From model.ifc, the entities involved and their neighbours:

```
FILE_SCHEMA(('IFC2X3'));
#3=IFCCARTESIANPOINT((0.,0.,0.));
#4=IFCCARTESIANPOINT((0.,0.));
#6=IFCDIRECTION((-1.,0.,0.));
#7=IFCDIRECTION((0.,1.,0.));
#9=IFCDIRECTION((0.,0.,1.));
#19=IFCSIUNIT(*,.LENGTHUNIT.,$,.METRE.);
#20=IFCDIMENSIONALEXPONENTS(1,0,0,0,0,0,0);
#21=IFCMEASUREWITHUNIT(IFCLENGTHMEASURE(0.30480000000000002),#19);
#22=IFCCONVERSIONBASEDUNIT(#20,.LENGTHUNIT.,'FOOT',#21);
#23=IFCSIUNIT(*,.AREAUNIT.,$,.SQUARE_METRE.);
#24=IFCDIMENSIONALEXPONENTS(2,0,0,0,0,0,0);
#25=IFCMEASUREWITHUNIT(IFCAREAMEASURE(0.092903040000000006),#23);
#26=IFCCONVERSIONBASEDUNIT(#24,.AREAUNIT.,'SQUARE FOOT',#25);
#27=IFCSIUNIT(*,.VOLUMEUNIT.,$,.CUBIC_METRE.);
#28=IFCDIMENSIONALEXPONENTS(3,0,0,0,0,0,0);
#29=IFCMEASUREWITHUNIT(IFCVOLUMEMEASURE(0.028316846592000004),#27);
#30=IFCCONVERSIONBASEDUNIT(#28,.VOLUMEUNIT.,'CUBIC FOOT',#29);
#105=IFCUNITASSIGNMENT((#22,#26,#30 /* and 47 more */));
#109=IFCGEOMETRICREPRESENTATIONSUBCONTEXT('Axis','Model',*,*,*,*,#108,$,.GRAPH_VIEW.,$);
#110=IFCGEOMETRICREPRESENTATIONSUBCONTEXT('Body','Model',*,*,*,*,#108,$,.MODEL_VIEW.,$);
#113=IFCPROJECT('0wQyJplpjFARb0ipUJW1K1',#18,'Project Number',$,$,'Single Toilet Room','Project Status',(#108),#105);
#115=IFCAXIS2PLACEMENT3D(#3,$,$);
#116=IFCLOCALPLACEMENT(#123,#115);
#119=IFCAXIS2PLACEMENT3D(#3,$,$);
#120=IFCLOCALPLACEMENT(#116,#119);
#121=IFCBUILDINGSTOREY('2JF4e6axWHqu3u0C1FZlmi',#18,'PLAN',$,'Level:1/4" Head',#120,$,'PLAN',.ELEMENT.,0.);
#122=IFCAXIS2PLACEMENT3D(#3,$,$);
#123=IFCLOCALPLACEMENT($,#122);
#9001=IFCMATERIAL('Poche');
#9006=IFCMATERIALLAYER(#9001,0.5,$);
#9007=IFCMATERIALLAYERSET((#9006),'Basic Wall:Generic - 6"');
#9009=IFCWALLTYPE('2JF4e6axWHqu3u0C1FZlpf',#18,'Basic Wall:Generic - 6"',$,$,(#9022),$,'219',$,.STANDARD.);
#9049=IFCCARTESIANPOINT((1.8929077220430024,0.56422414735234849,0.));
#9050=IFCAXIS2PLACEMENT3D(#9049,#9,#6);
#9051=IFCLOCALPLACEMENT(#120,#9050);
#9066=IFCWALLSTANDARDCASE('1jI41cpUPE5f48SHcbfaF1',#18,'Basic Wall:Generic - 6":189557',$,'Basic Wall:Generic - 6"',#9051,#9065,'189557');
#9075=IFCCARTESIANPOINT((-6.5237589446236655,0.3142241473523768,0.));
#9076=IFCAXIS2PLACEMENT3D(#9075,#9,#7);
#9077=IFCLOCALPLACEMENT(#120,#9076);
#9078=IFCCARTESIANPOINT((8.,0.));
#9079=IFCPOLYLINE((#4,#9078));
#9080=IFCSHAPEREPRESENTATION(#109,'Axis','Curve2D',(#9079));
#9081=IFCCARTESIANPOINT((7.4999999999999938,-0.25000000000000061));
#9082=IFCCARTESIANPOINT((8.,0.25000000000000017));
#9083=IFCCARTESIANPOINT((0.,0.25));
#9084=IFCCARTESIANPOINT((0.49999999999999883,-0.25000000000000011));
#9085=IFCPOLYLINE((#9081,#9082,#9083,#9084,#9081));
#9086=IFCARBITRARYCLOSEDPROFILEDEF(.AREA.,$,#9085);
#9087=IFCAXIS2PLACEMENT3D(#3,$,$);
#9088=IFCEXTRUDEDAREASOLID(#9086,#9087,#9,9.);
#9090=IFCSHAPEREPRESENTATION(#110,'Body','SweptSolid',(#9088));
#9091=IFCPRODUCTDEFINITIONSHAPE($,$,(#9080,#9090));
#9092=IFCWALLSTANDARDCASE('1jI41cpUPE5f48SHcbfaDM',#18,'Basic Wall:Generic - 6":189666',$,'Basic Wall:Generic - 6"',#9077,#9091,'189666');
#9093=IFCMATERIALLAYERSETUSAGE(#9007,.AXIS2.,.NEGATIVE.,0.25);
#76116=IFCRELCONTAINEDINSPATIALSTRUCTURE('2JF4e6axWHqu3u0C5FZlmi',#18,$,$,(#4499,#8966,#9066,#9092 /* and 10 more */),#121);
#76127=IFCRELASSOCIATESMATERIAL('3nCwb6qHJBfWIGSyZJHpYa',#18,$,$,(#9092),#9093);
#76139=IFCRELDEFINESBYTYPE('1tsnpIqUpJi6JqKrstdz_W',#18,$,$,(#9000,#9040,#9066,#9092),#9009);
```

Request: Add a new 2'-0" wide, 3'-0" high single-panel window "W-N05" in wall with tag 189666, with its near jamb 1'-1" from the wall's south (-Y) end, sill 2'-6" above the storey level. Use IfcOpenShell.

```python
import numpy as np
import ifcopenshell
import ifcopenshell.api.feature
import ifcopenshell.api.geometry
import ifcopenshell.api.root
import ifcopenshell.api.spatial
import ifcopenshell.api.type
import ifcopenshell.geom
import ifcopenshell.util.element
import ifcopenshell.util.placement
import ifcopenshell.util.representation
import ifcopenshell.util.shape
import ifcopenshell.util.unit

model = ifcopenshell.open("model.ifc")
unit_scale = ifcopenshell.util.unit.calculate_unit_scale(model)
settings = ifcopenshell.geom.settings()


def volume(element):
    """Net volume in cubic metres, openings subtracted."""
    shape = ifcopenshell.geom.create_shape(settings, element)
    return ifcopenshell.util.shape.get_volume(shape.geometry)


wall = model.by_id(9092)
storey = ifcopenshell.util.element.get_container(wall, ifc_class="IfcBuildingStorey")
context = ifcopenshell.util.representation.get_context(model, "Model", "Body", "MODEL_VIEW")
before = volume(wall)

width, height, from_end, sill = 0.6096, 0.9144, 0.3302, 0.762  # metres

# The wall runs along its own X axis, and the end named is its -X end.
wall_shape = ifcopenshell.geom.create_shape(settings, wall)
x, y, z = ifcopenshell.util.shape.get_vertices(wall_shape.geometry).T
start = x.min() + from_end
face, thickness = float(y.min()), float(y.max() - y.min())
wall_matrix = ifcopenshell.util.placement.get_local_placement(wall.ObjectPlacement)
level = ifcopenshell.util.placement.get_local_placement(storey.ObjectPlacement)[2, 3]


def in_wall(x, y):
    """Placement at x, y metres in the wall's axes, at sill height."""
    matrix = wall_matrix.copy()
    matrix[:, 3] = wall_matrix @ np.array([x / unit_scale, y / unit_scale, 0.0, 1.0])
    matrix[2, 3] = level + sill / unit_scale
    return matrix


# Opening: a box that overshoots both wall faces by 50 mm.
opening = ifcopenshell.api.root.create_entity(model, ifc_class="IfcOpeningElement")
box = ifcopenshell.api.geometry.add_wall_representation(
    model, context=context, length=width, height=height, thickness=thickness + 0.1
)
ifcopenshell.api.geometry.assign_representation(model, product=opening, representation=box)
ifcopenshell.api.geometry.edit_object_placement(model, product=opening, matrix=in_wall(start, face - 0.05), is_si=False)
ifcopenshell.api.feature.add_feature(model, feature=opening, element=wall)

window = ifcopenshell.api.root.create_entity(model, ifc_class="IfcWindow", name="W-N05")
window.OverallWidth, window.OverallHeight = width / unit_scale, height / unit_scale
body = ifcopenshell.api.geometry.add_window_representation(
    model,
    context=context,
    overall_width=window.OverallWidth,
    overall_height=window.OverallHeight,
    partition_type="SINGLE_PANEL",
)
ifcopenshell.api.geometry.assign_representation(model, product=window, representation=body)
ifcopenshell.api.spatial.assign_container(model, products=[window], relating_structure=storey)
fills = ifcopenshell.api.feature.add_filling(model, opening=opening, element=window)
fills.OwnerHistory = window.OwnerHistory  # required in IFC2X3

# IFC2X3 keeps the operation on the window style.
style = ifcopenshell.api.root.create_entity(model, ifc_class="IfcWindowStyle", name="W-N05")
style.OperationType, style.ConstructionType = "SINGLE_PANEL", "NOTDEFINED"
style.ParameterTakesPrecedence = style.Sizeable = False
ifcopenshell.api.type.assign_type(model, related_objects=[window], relating_type=style)

# Centre the window in the wall's thickness.
ifcopenshell.api.geometry.edit_object_placement(model, product=window, matrix=in_wall(start, face), is_si=False)
window_shape = ifcopenshell.geom.create_shape(settings, window)
depth = ifcopenshell.util.shape.get_vertices(window_shape.geometry)[:, 1]
offset = face + thickness / 2 - (depth.min() + depth.max()) / 2
ifcopenshell.api.geometry.edit_object_placement(model, product=window, matrix=in_wall(start, offset), is_si=False)

after = volume(wall)

print(f"wall volume {before:.3f} -> {after:.3f} m3")

model.write("model-out.ifc")
```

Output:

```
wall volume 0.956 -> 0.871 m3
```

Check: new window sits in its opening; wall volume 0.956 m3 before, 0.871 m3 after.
